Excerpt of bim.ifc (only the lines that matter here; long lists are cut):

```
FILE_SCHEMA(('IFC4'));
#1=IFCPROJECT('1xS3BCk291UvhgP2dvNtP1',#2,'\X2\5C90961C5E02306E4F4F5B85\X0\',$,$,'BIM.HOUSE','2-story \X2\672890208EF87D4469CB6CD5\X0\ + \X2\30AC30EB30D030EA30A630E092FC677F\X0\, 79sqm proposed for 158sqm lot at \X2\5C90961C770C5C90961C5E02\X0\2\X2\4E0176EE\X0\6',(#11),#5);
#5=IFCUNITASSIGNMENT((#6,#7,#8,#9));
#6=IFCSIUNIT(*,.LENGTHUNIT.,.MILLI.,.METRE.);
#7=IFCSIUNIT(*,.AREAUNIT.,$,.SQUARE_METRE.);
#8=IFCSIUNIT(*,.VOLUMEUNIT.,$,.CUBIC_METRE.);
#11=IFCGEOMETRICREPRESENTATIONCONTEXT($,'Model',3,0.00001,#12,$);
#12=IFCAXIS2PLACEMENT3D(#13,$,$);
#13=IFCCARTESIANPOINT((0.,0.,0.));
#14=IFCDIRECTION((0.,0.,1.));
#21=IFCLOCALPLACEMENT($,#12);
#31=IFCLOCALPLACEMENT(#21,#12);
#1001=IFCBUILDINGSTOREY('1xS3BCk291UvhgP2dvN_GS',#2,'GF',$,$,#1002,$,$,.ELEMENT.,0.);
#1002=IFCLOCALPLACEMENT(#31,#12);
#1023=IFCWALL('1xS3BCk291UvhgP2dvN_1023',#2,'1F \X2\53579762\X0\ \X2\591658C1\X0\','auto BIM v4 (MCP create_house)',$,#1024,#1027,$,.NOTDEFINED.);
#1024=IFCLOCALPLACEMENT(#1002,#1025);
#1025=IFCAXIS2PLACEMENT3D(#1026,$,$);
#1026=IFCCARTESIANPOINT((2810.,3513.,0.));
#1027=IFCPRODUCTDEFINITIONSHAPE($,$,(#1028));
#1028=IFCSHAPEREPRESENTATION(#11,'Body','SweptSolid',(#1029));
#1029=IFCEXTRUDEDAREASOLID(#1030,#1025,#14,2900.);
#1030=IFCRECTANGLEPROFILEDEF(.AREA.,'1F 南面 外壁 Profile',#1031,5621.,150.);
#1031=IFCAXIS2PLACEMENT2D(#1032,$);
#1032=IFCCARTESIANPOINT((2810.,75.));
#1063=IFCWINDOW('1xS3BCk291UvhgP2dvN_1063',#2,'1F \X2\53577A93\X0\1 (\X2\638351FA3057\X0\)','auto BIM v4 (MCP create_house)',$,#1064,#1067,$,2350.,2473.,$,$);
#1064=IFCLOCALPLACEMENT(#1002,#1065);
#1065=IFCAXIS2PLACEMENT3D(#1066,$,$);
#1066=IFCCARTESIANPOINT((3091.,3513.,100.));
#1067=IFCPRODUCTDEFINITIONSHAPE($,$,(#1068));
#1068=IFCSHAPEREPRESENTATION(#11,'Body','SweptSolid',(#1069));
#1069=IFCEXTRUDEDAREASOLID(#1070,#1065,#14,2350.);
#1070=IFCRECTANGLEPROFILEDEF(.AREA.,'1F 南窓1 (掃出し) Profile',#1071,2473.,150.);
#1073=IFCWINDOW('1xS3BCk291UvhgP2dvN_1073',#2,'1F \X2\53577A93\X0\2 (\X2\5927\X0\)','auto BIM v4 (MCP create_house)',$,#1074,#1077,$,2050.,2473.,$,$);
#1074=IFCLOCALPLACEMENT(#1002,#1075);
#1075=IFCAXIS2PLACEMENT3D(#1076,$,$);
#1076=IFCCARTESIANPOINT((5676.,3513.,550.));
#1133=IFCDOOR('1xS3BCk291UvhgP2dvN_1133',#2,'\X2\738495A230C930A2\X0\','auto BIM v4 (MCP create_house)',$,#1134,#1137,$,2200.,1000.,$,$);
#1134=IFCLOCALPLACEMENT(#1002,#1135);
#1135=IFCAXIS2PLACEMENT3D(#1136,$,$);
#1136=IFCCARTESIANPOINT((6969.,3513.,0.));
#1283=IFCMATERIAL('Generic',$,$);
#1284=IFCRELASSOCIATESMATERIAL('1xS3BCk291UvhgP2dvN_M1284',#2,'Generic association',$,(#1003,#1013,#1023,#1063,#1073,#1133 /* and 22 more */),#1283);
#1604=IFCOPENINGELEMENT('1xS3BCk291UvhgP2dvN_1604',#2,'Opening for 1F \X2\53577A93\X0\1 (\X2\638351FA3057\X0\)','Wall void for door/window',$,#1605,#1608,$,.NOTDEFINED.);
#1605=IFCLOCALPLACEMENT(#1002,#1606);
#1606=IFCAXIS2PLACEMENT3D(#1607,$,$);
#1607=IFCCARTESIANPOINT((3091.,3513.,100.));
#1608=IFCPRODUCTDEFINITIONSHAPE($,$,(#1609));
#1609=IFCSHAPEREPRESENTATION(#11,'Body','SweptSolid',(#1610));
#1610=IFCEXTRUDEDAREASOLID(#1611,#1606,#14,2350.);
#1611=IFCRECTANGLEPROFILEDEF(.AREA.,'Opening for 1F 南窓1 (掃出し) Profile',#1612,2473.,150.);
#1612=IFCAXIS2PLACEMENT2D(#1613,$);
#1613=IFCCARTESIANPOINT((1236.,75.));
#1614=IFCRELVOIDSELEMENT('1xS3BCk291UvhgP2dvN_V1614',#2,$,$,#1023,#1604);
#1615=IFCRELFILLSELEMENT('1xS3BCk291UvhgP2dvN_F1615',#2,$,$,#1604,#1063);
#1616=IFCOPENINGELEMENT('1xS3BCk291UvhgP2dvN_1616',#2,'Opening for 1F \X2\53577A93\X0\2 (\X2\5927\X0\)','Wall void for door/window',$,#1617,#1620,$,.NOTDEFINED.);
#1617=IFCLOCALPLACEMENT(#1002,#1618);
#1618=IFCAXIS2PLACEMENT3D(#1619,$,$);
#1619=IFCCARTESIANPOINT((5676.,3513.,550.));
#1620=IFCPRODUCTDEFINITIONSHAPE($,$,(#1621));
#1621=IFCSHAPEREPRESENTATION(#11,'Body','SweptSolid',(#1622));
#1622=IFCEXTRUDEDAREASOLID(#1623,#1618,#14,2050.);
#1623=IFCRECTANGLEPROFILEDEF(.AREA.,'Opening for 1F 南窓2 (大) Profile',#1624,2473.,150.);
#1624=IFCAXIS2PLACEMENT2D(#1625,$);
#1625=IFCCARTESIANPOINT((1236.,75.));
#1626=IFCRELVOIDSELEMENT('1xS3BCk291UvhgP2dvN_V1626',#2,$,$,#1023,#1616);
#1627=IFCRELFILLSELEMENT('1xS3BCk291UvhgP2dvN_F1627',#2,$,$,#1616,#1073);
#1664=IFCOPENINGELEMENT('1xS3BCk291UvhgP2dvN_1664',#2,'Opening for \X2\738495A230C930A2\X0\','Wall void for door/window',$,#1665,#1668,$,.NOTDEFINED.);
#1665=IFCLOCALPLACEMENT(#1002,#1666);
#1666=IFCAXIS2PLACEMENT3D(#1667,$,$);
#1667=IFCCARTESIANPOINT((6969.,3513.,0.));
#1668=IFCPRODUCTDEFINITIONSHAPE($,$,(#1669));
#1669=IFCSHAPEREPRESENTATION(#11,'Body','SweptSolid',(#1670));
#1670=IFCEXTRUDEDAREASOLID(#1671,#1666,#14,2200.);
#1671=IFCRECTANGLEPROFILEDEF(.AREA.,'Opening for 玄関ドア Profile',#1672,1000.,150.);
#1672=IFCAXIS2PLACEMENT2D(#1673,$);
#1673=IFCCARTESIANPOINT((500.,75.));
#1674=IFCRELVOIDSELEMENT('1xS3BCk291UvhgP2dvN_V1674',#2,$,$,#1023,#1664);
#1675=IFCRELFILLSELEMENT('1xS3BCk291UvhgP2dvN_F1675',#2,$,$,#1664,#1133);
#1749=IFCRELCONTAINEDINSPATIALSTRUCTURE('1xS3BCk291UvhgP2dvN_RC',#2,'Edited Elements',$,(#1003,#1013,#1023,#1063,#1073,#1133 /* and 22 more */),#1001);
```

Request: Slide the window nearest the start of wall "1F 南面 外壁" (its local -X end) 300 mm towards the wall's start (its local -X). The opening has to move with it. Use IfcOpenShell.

```python
import ifcopenshell
import ifcopenshell.api.geometry
import ifcopenshell.util.placement

model = ifcopenshell.open("bim.ifc")

window = model.by_guid("1xS3BCk291UvhgP2dvN_1063")
opening = window.FillsVoids[0].RelatingOpeningElement
wall = opening.VoidsElements[0].RelatingBuildingElement

wall_matrix = ifcopenshell.util.placement.get_local_placement(wall.ObjectPlacement)
shift = wall_matrix[:3, 0] * -300.0
before = ifcopenshell.util.placement.get_local_placement(window.ObjectPlacement)[:3, 3].copy()

# The window is not placed relative to its opening, so move both.
for product in (opening, window):
    matrix = ifcopenshell.util.placement.get_local_placement(product.ObjectPlacement)
    matrix[:3, 3] += shift
    ifcopenshell.api.geometry.edit_object_placement(model, product=product, matrix=matrix, is_si=False)

after = ifcopenshell.util.placement.get_local_placement(window.ObjectPlacement)[:3, 3]
print("window moved by", (after - before).round(3) + 0.0)

model.write("bim_v2.ifc")
```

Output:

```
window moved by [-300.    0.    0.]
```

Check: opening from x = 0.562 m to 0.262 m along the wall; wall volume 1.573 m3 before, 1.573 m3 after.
